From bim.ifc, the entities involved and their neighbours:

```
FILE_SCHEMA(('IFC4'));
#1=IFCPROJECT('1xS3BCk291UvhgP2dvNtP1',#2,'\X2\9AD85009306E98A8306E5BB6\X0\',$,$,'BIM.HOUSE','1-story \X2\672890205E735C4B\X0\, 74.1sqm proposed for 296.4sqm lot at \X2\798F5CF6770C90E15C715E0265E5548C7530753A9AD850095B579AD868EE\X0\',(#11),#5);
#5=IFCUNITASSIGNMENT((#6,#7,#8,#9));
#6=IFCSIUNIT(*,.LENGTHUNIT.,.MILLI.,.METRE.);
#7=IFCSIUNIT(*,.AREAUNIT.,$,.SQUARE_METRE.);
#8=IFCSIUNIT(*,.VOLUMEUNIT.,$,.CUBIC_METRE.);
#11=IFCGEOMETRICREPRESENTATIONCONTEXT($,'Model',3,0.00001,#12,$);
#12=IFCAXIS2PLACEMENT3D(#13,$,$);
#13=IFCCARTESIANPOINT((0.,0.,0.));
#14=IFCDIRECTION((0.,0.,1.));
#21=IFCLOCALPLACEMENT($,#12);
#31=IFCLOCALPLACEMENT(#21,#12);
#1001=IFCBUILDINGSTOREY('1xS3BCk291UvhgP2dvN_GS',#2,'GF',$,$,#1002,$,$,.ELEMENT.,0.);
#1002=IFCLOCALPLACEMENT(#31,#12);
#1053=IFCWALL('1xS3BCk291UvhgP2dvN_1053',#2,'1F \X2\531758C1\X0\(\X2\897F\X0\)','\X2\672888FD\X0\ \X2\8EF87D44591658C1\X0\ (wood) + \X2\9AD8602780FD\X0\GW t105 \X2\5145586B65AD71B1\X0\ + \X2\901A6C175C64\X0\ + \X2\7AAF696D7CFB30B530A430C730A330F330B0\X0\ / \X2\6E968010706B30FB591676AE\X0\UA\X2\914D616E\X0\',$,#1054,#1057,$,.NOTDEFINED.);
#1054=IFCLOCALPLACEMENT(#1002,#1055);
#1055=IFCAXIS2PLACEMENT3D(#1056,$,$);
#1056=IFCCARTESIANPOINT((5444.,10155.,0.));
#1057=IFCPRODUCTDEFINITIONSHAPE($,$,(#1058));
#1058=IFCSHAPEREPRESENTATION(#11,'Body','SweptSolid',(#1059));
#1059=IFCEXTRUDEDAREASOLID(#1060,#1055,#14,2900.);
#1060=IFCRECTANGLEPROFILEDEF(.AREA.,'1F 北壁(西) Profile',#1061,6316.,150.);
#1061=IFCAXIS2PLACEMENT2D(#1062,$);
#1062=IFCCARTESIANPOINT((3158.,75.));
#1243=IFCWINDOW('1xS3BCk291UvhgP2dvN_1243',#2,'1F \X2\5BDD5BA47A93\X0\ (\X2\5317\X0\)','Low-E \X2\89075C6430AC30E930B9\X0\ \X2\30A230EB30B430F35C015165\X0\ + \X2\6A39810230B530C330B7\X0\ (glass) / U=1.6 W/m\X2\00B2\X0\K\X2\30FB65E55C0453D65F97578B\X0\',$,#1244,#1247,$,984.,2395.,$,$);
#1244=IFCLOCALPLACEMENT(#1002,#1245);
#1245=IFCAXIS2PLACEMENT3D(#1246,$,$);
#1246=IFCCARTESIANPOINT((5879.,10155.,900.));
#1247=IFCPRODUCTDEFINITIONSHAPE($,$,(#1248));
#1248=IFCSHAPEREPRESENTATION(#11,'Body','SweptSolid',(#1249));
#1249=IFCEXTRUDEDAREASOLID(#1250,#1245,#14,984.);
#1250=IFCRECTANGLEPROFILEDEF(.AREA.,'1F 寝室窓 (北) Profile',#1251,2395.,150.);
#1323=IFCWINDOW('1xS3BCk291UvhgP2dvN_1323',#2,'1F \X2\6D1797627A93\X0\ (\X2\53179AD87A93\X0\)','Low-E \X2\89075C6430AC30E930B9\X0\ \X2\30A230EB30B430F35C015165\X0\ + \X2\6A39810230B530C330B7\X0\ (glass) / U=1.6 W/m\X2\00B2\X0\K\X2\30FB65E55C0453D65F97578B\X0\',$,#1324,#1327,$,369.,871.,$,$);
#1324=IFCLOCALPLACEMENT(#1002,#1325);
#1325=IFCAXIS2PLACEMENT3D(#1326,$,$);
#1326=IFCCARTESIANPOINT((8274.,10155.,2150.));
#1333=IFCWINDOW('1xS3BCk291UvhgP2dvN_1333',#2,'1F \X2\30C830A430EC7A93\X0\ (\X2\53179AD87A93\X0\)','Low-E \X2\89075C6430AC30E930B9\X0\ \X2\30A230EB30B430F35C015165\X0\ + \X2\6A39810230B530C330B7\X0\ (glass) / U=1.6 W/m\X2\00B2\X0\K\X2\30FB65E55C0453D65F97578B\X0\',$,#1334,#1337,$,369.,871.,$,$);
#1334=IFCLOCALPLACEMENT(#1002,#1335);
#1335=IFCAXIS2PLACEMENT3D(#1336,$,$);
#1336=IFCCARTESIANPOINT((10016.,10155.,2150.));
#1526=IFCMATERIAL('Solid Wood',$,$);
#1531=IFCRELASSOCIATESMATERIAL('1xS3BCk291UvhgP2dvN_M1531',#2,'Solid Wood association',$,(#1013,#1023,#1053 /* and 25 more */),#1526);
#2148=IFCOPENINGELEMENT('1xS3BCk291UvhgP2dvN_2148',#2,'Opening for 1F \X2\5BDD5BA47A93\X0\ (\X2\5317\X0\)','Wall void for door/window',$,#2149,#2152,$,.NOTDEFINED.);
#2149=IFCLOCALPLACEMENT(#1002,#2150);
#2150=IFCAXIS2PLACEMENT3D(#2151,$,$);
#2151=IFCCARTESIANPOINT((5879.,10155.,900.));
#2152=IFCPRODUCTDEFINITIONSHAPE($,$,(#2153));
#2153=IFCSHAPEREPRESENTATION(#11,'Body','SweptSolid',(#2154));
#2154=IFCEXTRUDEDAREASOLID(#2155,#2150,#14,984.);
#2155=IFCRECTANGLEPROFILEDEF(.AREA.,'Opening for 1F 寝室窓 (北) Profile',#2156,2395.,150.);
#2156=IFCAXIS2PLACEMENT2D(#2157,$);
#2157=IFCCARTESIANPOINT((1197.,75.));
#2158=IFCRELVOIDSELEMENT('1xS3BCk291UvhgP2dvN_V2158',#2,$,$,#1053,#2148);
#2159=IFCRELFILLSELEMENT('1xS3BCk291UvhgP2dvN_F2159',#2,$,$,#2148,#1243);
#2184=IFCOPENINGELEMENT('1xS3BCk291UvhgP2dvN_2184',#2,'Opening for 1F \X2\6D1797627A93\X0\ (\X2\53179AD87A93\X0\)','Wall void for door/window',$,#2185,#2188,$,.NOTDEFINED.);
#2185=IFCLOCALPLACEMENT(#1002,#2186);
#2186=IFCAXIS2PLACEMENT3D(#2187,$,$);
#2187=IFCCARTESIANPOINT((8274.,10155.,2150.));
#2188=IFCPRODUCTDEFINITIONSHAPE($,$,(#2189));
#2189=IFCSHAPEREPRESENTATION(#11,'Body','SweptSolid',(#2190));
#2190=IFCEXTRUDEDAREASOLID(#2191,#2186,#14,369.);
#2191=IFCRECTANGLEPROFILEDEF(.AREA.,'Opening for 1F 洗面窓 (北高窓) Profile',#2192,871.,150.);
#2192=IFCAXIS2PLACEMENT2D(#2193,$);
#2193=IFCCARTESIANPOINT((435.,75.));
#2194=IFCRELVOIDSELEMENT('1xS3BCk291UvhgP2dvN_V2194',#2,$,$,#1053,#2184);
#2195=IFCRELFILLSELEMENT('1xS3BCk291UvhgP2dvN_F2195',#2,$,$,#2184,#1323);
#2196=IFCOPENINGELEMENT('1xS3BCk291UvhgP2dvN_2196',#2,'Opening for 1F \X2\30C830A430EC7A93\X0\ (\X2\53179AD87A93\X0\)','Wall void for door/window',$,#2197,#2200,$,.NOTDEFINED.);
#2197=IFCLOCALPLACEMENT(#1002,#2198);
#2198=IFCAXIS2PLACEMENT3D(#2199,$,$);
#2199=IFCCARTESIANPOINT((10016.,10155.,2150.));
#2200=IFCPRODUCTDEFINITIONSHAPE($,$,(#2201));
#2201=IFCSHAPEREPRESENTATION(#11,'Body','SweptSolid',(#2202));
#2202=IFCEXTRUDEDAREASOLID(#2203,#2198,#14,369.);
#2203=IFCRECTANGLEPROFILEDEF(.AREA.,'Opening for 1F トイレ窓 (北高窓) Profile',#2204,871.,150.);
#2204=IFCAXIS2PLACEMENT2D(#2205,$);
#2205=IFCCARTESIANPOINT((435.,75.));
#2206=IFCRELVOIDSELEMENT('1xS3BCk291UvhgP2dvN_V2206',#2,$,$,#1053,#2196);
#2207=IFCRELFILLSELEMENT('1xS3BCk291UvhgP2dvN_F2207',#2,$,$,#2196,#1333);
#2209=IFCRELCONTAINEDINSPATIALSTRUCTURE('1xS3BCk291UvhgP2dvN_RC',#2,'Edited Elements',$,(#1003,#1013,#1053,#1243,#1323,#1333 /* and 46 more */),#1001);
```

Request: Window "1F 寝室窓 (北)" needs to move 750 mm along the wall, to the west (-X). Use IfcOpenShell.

```python
import ifcopenshell
import ifcopenshell.api.geometry
import ifcopenshell.util.placement

model = ifcopenshell.open("bim.ifc")

window = model.by_id(1243)
opening = window.FillsVoids[0].RelatingOpeningElement
wall = opening.VoidsElements[0].RelatingBuildingElement

wall_matrix = ifcopenshell.util.placement.get_local_placement(wall.ObjectPlacement)
shift = wall_matrix[:3, 0] * -750.0
before = ifcopenshell.util.placement.get_local_placement(window.ObjectPlacement)[:3, 3].copy()

# The window is not placed relative to its opening, so move both.
for product in (opening, window):
    matrix = ifcopenshell.util.placement.get_local_placement(product.ObjectPlacement)
    matrix[:3, 3] += shift
    ifcopenshell.api.geometry.edit_object_placement(model, product=product, matrix=matrix, is_si=False)

after = ifcopenshell.util.placement.get_local_placement(window.ObjectPlacement)[:3, 3]
print("window moved by", (after - before).round(3) + 0.0)

model.write("bim_rev.ifc")
```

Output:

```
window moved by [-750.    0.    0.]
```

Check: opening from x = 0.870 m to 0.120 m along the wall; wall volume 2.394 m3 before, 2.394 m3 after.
